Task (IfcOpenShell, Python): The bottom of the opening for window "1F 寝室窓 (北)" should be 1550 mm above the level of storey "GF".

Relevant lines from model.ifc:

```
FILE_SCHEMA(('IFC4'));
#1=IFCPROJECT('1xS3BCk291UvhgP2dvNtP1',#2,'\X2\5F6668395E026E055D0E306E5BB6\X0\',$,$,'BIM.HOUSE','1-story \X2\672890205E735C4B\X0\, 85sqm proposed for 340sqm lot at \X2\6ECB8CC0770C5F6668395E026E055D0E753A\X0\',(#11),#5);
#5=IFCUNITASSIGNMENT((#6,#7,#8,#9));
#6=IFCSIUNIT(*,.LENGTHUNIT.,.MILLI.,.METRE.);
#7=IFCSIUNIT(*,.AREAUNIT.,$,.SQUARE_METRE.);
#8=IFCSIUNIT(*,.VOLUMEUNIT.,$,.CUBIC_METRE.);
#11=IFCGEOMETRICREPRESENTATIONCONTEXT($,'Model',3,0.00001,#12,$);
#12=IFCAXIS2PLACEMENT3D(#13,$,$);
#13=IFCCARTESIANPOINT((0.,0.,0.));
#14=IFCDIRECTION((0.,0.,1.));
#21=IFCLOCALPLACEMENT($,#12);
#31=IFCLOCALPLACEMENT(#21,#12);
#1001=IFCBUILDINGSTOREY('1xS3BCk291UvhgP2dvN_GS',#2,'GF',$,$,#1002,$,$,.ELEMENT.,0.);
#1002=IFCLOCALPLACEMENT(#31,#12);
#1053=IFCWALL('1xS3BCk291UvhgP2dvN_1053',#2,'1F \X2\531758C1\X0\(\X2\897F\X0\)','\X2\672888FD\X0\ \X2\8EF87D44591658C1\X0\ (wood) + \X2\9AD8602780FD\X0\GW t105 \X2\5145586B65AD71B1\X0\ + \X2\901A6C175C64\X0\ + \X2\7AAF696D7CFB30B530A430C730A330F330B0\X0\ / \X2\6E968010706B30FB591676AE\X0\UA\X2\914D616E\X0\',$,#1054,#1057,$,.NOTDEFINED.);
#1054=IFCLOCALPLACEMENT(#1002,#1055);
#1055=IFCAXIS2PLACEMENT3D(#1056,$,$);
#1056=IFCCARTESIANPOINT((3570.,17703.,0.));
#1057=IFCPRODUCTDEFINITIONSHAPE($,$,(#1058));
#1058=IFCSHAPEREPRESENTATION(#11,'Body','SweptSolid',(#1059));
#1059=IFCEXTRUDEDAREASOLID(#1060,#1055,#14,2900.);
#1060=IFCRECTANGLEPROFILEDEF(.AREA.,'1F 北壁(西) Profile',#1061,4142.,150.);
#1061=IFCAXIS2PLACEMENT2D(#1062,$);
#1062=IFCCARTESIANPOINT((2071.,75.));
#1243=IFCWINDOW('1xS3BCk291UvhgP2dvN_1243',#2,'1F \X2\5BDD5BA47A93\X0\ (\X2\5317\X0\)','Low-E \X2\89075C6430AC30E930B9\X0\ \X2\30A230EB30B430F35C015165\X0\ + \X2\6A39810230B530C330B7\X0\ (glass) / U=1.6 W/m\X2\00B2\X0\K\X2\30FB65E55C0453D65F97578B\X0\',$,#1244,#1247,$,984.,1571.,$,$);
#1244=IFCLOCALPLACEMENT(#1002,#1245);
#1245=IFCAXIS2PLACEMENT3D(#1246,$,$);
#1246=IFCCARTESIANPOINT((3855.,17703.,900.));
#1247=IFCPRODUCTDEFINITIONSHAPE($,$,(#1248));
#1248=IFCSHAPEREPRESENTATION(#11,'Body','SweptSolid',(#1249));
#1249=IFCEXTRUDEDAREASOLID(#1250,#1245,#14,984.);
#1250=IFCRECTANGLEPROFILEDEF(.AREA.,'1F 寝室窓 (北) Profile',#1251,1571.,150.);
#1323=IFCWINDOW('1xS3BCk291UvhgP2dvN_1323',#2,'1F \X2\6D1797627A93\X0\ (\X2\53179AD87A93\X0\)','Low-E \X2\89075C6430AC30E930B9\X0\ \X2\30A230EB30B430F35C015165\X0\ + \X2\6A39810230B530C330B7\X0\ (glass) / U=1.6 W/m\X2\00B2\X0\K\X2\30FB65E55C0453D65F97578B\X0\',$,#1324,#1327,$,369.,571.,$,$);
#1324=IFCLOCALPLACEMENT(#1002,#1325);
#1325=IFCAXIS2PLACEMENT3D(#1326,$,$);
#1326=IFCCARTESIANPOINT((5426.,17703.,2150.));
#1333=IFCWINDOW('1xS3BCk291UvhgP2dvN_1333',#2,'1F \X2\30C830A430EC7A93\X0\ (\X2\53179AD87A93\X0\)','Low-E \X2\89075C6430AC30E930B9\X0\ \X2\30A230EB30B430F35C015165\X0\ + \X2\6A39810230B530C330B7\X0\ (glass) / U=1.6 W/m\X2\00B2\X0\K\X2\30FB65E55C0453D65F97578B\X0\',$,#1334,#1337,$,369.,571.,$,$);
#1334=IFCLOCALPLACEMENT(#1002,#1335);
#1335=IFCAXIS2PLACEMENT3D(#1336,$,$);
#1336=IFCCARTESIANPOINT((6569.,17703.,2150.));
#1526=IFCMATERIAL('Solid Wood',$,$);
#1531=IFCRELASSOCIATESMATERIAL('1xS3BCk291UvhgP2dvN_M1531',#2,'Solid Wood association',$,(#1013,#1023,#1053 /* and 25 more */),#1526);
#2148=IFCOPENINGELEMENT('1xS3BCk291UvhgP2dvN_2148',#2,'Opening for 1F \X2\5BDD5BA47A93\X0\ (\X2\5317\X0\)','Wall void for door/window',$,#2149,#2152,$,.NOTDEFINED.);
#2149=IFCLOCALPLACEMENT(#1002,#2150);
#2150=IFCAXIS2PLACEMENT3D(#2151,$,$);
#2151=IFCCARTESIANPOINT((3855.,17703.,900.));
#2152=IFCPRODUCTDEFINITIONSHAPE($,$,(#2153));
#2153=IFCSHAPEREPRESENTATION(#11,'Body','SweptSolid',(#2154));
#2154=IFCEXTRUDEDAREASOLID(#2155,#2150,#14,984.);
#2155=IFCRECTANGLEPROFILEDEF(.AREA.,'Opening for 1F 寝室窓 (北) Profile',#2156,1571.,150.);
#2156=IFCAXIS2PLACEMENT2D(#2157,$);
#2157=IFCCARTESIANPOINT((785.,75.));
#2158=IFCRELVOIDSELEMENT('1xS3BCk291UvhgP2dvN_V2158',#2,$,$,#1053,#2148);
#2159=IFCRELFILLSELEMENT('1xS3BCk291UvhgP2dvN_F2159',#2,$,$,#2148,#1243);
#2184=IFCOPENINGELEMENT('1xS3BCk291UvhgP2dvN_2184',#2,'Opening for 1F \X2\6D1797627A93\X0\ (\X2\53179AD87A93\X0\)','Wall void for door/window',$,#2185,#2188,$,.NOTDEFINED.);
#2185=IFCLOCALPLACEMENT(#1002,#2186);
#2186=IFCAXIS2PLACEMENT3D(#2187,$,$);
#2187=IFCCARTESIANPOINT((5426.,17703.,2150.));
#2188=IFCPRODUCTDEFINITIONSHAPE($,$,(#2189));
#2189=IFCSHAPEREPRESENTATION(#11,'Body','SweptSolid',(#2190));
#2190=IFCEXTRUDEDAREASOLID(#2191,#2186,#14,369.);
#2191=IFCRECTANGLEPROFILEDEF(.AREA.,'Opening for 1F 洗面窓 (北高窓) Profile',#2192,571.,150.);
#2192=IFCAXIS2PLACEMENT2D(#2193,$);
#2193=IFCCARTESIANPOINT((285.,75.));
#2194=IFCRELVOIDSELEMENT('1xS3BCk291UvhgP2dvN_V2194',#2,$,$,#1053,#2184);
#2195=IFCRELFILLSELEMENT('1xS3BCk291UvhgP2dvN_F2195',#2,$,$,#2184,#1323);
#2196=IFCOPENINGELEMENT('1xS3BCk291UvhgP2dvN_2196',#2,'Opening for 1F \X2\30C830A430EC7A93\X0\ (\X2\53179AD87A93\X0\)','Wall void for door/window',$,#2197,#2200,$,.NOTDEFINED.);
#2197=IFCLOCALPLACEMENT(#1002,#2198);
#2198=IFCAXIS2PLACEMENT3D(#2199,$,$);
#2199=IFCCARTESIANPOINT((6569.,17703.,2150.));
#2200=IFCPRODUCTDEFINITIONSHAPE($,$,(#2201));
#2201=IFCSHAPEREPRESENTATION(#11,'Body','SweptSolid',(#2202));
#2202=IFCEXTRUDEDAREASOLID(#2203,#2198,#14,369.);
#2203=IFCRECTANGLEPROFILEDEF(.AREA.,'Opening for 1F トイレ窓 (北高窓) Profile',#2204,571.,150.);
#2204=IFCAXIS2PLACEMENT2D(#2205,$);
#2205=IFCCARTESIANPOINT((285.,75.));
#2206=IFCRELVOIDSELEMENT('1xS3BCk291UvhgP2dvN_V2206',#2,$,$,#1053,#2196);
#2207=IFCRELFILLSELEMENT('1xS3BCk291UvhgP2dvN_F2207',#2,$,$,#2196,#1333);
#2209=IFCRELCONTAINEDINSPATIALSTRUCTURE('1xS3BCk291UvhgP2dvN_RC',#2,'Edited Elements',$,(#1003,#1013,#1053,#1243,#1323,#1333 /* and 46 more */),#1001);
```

```python
import numpy as np
import ifcopenshell
import ifcopenshell.api.geometry
import ifcopenshell.geom
import ifcopenshell.util.element
import ifcopenshell.util.placement
import ifcopenshell.util.shape
import ifcopenshell.util.unit

model = ifcopenshell.open("model.ifc")
unit_scale = ifcopenshell.util.unit.calculate_unit_scale(model)

window = model.by_id(1243)
opening = window.FillsVoids[0].RelatingOpeningElement
storey = ifcopenshell.util.element.get_container(window, ifc_class="IfcBuildingStorey")
level = ifcopenshell.util.placement.get_local_placement(storey.ObjectPlacement)[2, 3]

# The opening's origin need not be at the sill, so measure its lowest point.
shape = ifcopenshell.geom.create_shape(ifcopenshell.geom.settings(), opening)
bottom = ifcopenshell.util.shape.get_shape_bottom_elevation(shape, shape.geometry) / unit_scale
dz = level + 1550.0 - bottom

shift = np.array([0.0, 0.0, dz])
# The window is not placed relative to its opening, so move both.
for product in (opening, window):
    matrix = ifcopenshell.util.placement.get_local_placement(product.ObjectPlacement)
    matrix[:3, 3] += shift
    ifcopenshell.api.geometry.edit_object_placement(model, product=product, matrix=matrix, is_si=False)

print(f"moved by {dz * unit_scale:+.3f} m")

model.write("model_v2.ifc")
```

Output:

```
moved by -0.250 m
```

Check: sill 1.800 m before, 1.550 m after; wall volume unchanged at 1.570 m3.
